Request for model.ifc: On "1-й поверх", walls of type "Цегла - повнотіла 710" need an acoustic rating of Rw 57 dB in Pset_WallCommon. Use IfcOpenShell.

First a look at what the model holds.

```python
import ifcopenshell
import ifcopenshell.util.element

model = ifcopenshell.open("model.ifc")
print(model.schema)
storey = next(s for s in model.by_type("IfcBuildingStorey") if s.Name == "1-й поверх")
walls = [e for e in ifcopenshell.util.element.get_decomposition(storey) if e.is_a("IfcWall")]
seen = {}
for e in walls:
    element_type = ifcopenshell.util.element.get_type(e)
    key = (element_type.Name if element_type != e and element_type else None, ifcopenshell.util.element.get_pset(e, "Pset_WallCommon", "AcousticRating"))
    seen[key] = seen.get(key, 0) + 1
for (name, value), count in sorted(seen.items(), key=str):
    print(count, "x", name, "|", value)
```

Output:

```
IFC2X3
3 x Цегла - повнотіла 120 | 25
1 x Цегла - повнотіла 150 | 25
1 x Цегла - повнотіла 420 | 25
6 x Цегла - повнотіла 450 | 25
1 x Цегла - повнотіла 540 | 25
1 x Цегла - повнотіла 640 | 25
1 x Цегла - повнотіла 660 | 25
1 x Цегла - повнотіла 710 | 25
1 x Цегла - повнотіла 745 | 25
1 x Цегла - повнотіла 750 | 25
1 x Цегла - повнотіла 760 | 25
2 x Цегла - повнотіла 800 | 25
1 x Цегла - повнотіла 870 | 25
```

```python
import ifcopenshell
import ifcopenshell.api.pset
import ifcopenshell.util.element

model = ifcopenshell.open("model.ifc")

storey = next(s for s in model.by_type("IfcBuildingStorey") if s.Name == "1-й поверх")
walls = [e for e in ifcopenshell.util.element.get_decomposition(storey) if e.is_a("IfcWall")]

count = 0
for e in walls:
    element_type = ifcopenshell.util.element.get_type(e)
    if element_type in (None, e) or element_type.Name != "Цегла - повнотіла 710":
        continue
    # add_pset returns the element's existing set when there is one.
    pset = ifcopenshell.api.pset.add_pset(model, product=e, name="Pset_WallCommon")
    ifcopenshell.api.pset.edit_pset(model, pset=pset, properties={"AcousticRating": "Rw 57 dB"})
    count += 1

print(count, "walls updated")

model.write("model_rev.ifc")
```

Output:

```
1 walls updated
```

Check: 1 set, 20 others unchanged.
